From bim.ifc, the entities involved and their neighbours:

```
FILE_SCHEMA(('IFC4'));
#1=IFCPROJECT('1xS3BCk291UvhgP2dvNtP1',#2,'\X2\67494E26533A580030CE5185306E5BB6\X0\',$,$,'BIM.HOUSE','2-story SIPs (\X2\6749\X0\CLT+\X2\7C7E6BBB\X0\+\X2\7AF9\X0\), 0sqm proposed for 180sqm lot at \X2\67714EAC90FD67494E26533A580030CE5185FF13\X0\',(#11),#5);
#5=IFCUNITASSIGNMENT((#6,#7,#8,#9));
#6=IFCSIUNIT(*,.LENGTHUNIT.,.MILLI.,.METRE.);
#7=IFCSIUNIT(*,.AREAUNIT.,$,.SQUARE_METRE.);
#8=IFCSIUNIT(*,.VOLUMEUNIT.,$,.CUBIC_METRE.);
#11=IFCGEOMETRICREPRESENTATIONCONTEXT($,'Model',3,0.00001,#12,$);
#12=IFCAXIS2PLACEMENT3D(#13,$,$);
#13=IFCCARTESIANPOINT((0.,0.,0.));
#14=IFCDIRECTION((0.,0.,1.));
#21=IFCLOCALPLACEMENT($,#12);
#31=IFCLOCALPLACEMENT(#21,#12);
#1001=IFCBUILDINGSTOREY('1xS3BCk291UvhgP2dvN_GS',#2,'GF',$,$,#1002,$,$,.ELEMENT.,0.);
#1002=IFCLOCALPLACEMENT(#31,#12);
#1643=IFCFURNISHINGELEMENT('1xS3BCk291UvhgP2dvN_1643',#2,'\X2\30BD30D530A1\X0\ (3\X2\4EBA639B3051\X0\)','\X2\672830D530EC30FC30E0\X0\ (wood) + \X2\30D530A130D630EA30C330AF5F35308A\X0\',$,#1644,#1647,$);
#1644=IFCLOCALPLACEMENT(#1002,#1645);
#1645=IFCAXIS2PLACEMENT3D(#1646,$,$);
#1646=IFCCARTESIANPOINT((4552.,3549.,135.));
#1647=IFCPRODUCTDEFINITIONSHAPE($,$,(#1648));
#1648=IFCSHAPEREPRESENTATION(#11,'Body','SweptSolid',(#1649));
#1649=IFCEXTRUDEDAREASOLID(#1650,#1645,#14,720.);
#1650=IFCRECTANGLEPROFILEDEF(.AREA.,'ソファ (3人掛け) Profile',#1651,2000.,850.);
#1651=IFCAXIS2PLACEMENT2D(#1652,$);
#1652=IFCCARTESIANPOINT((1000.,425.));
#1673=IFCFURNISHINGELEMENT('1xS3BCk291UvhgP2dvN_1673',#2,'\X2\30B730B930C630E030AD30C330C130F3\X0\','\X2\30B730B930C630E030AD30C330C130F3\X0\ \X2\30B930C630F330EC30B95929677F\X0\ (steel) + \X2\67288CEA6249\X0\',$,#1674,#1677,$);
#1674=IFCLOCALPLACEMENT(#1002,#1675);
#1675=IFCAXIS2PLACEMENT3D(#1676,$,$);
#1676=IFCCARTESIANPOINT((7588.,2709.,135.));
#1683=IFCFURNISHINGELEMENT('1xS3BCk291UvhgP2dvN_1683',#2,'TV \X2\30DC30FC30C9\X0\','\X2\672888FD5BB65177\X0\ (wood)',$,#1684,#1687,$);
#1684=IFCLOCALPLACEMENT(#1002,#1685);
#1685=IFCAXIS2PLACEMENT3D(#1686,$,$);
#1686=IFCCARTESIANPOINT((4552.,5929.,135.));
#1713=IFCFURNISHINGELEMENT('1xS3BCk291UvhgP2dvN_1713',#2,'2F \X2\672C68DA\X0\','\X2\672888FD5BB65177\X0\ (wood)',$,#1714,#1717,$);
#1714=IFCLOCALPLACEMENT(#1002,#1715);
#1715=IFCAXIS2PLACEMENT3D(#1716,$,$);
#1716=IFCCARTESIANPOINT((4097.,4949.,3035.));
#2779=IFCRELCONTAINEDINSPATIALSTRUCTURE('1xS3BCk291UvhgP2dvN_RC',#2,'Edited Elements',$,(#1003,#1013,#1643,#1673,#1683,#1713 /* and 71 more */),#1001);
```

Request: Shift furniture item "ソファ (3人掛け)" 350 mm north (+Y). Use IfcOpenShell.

```python
import ifcopenshell
import ifcopenshell.api.geometry
import ifcopenshell.util.placement
import ifcopenshell.util.unit

model = ifcopenshell.open("bim.ifc")
unit_scale = ifcopenshell.util.unit.calculate_unit_scale(model)

item = model.by_guid("1xS3BCk291UvhgP2dvN_1643")
matrix = ifcopenshell.util.placement.get_local_placement(item.ObjectPlacement)
matrix[1, 3] += 0.35 / unit_scale
ifcopenshell.api.geometry.edit_object_placement(model, product=item, matrix=matrix, is_si=False)

print(ifcopenshell.util.placement.get_local_placement(item.ObjectPlacement).round(3) + 0.0)

model.write("bim_edited.ifc")
```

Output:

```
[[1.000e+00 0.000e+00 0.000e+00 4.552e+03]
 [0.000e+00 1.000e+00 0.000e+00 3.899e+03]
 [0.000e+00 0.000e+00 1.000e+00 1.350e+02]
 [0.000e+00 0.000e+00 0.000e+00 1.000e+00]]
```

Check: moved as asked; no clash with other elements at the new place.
